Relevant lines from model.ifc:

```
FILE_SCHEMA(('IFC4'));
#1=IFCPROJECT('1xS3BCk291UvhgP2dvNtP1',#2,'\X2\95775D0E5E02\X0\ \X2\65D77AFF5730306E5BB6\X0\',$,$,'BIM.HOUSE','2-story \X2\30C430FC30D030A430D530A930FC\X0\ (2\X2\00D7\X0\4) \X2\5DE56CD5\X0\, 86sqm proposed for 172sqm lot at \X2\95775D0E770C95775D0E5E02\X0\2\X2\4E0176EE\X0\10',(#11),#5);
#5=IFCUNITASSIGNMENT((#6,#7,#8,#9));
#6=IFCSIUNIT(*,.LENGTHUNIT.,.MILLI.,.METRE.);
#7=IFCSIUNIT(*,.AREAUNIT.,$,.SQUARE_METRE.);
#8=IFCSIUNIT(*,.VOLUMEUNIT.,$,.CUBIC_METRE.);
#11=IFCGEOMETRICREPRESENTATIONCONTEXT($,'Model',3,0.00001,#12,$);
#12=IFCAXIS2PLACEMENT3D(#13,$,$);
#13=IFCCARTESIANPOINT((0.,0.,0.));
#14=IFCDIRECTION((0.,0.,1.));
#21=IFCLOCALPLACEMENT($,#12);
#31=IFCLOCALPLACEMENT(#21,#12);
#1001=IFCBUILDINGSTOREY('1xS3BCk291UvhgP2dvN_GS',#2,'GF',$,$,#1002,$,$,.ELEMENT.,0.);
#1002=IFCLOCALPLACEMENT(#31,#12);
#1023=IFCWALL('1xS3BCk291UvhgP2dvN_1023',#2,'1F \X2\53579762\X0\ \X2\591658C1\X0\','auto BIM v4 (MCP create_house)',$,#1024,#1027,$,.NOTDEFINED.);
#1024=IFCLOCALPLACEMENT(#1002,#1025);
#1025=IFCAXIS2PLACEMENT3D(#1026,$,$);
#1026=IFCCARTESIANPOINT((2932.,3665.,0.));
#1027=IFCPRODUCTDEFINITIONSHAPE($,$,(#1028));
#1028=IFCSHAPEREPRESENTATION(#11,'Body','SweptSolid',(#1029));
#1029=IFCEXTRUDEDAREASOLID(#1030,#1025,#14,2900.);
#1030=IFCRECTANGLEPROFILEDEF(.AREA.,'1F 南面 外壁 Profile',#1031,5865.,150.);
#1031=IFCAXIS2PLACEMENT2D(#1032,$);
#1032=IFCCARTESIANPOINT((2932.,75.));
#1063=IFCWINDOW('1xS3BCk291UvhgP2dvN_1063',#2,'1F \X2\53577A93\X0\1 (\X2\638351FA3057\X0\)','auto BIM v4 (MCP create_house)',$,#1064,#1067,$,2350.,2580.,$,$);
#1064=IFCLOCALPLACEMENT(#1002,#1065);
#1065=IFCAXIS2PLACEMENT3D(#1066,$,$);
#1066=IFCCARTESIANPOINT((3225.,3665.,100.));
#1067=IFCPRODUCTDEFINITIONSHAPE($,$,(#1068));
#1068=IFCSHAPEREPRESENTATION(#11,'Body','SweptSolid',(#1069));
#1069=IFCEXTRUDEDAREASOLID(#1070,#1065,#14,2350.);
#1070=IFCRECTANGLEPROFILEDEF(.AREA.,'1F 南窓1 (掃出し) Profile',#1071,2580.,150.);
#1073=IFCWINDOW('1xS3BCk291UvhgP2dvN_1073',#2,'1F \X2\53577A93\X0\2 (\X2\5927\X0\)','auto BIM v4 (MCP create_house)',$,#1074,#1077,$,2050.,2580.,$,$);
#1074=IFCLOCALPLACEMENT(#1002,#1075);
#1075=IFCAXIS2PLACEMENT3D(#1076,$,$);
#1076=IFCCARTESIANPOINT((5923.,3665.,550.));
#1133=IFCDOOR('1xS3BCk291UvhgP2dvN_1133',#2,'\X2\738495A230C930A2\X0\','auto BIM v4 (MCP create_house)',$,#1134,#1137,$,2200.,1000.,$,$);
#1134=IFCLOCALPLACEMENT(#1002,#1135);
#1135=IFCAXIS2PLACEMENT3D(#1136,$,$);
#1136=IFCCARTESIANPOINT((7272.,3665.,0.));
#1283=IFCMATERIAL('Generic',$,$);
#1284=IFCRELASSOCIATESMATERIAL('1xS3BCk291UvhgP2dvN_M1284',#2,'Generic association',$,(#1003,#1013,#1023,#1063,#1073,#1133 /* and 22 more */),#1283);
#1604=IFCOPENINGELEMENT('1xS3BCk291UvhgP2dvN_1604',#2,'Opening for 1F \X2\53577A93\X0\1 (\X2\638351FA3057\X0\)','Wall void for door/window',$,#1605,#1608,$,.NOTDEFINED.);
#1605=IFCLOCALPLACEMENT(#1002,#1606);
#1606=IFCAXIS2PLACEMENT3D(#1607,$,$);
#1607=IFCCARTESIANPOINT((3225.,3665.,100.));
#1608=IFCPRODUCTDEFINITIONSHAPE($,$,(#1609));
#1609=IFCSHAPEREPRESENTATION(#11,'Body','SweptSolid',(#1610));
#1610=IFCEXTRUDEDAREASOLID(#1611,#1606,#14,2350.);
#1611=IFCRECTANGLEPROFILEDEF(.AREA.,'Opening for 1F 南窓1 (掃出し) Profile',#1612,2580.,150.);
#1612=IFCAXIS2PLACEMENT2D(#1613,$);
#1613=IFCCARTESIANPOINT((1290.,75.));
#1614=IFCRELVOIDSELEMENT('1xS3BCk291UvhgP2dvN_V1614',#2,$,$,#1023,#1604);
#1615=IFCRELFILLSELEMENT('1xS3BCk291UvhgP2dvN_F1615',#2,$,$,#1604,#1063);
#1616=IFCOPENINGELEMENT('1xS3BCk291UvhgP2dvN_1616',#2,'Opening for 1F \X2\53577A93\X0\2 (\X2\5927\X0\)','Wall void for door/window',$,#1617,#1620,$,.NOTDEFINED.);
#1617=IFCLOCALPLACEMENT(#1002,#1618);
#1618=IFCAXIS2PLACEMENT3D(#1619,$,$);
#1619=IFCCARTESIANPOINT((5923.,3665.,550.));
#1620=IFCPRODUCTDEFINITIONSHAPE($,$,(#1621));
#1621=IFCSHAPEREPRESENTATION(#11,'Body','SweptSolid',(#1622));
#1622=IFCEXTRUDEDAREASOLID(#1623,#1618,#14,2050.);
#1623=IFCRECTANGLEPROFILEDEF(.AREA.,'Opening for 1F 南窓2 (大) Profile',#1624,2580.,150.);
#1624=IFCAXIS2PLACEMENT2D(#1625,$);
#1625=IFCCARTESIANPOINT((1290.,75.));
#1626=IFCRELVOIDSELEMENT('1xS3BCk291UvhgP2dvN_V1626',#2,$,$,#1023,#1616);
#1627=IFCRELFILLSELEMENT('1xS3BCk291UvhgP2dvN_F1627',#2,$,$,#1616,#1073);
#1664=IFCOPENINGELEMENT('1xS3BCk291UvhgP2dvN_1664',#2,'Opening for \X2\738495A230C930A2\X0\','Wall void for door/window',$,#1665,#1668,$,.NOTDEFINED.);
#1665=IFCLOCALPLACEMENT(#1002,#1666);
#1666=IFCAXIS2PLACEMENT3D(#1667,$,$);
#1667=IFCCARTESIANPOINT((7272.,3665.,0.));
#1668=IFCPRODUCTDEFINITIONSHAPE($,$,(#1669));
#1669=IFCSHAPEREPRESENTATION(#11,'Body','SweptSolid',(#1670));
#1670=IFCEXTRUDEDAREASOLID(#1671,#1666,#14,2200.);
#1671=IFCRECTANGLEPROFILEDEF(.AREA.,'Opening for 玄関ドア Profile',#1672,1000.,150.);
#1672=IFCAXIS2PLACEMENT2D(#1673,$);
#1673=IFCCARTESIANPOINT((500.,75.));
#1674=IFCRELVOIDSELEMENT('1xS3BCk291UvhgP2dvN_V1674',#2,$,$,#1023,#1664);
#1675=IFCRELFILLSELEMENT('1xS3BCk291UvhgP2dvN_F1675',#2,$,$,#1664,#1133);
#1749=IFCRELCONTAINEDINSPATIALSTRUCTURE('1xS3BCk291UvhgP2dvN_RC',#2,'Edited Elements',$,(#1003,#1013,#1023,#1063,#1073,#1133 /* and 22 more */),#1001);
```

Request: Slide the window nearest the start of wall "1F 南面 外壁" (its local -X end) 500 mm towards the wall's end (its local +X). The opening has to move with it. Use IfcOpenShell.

```python
import ifcopenshell
import ifcopenshell.api.geometry
import ifcopenshell.util.placement
import ifcopenshell.util.unit

model = ifcopenshell.open("model.ifc")
unit_scale = ifcopenshell.util.unit.calculate_unit_scale(model)

window = model.by_guid("1xS3BCk291UvhgP2dvN_1063")
opening = window.FillsVoids[0].RelatingOpeningElement
wall = opening.VoidsElements[0].RelatingBuildingElement

wall_matrix = ifcopenshell.util.placement.get_local_placement(wall.ObjectPlacement)
shift = wall_matrix[:3, 0] * 0.5 / unit_scale
before = ifcopenshell.util.placement.get_local_placement(window.ObjectPlacement)[:3, 3].copy()

# The window is not placed relative to its opening, so move both.
for product in (opening, window):
    matrix = ifcopenshell.util.placement.get_local_placement(product.ObjectPlacement)
    matrix[:3, 3] += shift
    ifcopenshell.api.geometry.edit_object_placement(model, product=product, matrix=matrix, is_si=False)

after = ifcopenshell.util.placement.get_local_placement(window.ObjectPlacement)[:3, 3]
print("window moved by", (after - before).round(3) + 0.0)

model.write("model_updated.ifc")
```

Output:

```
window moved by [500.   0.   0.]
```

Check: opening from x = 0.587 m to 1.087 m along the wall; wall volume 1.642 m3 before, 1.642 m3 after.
